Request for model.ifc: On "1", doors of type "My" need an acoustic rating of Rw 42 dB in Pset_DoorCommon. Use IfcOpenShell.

First a look at what the model holds.

```python
import ifcopenshell
import ifcopenshell.util.element

model = ifcopenshell.open("model.ifc")
print(model.schema)
storey = next(s for s in model.by_type("IfcBuildingStorey") if s.Name == "1")
doors = [e for e in ifcopenshell.util.element.get_decomposition(storey) if e.is_a("IfcDoor")]
seen = {}
for e in doors:
    element_type = ifcopenshell.util.element.get_type(e)
    key = (element_type.Name if element_type != e and element_type else None, ifcopenshell.util.element.get_pset(e, "Pset_DoorCommon", "AcousticRating"))
    seen[key] = seen.get(key, 0) + 1
for (name, value), count in sorted(seen.items(), key=str):
    print(count, "x", name, "|", value)
```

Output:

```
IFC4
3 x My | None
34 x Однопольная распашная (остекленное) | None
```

```python
import ifcopenshell
import ifcopenshell.api.pset
import ifcopenshell.util.element

model = ifcopenshell.open("model.ifc")

storey = next(s for s in model.by_type("IfcBuildingStorey") if s.Name == "1")
doors = [e for e in ifcopenshell.util.element.get_decomposition(storey) if e.is_a("IfcDoor")]

count = 0
for e in doors:
    element_type = ifcopenshell.util.element.get_type(e)
    if element_type in (None, e) or element_type.Name != "My":
        continue
    # add_pset returns the element's existing set when there is one.
    pset = ifcopenshell.api.pset.add_pset(model, product=e, name="Pset_DoorCommon")
    ifcopenshell.api.pset.edit_pset(model, pset=pset, properties={"AcousticRating": "Rw 42 dB"})
    count += 1

print(count, "doors updated")

model.write("model_rev.ifc")
```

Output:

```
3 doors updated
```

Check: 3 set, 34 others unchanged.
